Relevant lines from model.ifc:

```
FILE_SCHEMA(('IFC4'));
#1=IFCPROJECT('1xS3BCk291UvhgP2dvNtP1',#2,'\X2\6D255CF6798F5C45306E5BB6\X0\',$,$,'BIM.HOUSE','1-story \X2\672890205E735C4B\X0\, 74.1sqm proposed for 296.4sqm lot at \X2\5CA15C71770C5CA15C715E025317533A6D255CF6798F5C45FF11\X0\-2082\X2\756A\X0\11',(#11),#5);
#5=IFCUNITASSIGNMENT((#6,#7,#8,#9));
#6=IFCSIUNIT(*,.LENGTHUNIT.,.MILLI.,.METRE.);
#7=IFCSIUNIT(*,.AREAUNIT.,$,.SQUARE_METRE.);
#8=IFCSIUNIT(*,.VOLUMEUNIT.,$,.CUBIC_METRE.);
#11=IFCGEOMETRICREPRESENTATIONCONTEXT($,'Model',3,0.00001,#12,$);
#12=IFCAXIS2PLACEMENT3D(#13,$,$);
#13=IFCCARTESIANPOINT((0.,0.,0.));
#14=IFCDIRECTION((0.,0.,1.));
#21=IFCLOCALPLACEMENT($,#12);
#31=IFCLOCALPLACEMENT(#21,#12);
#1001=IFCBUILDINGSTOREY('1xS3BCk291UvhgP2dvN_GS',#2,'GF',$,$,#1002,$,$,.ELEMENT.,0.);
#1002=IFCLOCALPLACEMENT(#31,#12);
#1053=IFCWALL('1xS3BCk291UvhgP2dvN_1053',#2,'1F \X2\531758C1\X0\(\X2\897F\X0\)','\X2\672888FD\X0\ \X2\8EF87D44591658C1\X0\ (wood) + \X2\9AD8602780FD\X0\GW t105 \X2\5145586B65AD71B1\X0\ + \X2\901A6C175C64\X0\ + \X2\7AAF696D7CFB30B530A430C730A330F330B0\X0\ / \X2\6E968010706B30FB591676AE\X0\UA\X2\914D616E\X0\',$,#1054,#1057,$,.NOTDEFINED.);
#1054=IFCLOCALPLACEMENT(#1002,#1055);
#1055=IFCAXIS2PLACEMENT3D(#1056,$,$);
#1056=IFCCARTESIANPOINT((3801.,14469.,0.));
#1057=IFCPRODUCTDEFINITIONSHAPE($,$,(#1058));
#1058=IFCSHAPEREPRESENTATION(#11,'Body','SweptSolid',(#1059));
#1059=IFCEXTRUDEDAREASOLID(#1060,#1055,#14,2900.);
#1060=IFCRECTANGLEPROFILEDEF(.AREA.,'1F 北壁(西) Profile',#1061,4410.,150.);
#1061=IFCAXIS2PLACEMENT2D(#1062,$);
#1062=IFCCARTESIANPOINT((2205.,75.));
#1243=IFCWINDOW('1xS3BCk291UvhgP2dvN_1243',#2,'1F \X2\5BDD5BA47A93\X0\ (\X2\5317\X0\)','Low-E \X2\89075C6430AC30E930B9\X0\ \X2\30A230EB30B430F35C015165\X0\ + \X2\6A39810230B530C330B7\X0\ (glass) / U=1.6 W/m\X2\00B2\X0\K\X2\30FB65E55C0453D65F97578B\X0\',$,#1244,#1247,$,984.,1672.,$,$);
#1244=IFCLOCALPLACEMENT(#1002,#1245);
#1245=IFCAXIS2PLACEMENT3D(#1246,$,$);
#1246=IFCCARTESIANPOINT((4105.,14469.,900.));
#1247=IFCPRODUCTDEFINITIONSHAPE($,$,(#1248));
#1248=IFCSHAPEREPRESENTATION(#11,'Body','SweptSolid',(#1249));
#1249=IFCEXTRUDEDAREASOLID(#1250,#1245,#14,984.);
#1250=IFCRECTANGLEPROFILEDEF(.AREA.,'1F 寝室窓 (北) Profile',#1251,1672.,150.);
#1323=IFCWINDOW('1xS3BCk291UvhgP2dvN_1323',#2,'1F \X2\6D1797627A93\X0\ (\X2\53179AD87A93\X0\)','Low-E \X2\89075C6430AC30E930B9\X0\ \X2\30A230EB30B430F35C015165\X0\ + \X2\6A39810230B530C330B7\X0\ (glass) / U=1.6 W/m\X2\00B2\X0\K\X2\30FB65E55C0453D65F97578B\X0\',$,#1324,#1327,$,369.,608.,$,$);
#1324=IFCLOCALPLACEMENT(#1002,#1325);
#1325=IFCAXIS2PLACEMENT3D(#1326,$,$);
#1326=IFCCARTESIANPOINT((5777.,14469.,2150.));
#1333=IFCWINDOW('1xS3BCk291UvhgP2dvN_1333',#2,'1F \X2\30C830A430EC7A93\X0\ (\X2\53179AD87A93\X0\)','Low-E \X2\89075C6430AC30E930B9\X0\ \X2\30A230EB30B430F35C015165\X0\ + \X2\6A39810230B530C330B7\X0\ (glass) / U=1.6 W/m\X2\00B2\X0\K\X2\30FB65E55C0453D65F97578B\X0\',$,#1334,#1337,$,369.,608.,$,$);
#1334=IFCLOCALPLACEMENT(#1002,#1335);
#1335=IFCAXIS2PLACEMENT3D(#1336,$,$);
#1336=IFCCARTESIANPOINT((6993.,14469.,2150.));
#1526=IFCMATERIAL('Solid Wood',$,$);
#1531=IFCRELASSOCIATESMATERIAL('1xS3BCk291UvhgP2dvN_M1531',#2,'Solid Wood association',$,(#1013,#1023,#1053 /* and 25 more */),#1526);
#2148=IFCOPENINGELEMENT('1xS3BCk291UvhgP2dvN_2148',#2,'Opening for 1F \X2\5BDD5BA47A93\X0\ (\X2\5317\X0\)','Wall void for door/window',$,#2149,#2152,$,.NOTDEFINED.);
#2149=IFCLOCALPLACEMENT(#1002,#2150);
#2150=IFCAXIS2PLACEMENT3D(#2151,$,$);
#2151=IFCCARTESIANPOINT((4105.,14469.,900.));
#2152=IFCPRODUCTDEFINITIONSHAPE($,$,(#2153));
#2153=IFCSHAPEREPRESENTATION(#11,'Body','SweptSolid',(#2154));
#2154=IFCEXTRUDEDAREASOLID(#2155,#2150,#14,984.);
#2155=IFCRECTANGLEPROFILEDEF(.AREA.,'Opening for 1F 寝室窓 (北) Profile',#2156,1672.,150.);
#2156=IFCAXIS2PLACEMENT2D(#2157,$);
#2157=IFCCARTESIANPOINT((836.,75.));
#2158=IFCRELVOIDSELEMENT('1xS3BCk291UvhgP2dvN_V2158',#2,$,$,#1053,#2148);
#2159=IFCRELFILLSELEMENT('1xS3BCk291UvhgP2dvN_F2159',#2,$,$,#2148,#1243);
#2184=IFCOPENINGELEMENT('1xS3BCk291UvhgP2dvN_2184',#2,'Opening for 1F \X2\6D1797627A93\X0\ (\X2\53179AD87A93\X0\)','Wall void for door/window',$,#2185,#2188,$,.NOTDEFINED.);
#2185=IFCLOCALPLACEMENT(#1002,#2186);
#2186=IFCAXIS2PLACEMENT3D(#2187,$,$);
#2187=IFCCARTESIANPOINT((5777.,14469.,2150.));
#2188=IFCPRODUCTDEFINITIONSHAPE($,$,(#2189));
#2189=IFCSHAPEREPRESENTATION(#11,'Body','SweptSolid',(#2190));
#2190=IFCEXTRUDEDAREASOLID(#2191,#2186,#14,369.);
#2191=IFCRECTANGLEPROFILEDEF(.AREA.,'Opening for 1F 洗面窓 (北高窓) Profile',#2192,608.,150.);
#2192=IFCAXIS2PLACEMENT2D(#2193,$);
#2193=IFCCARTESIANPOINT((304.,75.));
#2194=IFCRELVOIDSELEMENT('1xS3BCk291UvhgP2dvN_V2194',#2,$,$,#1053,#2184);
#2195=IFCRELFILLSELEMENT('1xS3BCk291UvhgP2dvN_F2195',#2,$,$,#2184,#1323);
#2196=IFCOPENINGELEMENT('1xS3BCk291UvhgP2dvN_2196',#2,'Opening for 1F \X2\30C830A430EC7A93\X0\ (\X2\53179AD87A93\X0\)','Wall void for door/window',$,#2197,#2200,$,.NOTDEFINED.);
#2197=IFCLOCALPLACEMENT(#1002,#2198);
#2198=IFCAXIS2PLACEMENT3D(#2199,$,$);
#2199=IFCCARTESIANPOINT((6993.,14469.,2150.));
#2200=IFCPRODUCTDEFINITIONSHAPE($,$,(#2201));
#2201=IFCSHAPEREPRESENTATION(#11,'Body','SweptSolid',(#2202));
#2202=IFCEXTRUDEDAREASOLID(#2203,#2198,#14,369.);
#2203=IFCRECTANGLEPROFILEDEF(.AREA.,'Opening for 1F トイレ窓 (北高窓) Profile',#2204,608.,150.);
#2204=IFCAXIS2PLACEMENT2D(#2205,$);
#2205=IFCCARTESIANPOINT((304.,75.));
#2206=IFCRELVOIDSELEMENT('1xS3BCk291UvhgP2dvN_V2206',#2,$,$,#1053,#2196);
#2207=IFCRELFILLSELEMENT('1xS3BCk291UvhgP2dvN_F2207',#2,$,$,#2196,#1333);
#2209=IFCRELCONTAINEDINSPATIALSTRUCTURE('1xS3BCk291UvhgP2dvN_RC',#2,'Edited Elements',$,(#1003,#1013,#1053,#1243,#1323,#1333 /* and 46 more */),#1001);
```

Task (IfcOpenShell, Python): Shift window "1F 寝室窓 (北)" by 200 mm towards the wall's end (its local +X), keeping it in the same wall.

```python
import ifcopenshell
import ifcopenshell.api.geometry
import ifcopenshell.util.placement
import ifcopenshell.util.unit

model = ifcopenshell.open("model.ifc")
unit_scale = ifcopenshell.util.unit.calculate_unit_scale(model)

window = model.by_id(1243)
opening = window.FillsVoids[0].RelatingOpeningElement
wall = opening.VoidsElements[0].RelatingBuildingElement

wall_matrix = ifcopenshell.util.placement.get_local_placement(wall.ObjectPlacement)
shift = wall_matrix[:3, 0] * 0.2 / unit_scale
before = ifcopenshell.util.placement.get_local_placement(window.ObjectPlacement)[:3, 3].copy()

# The window is not placed relative to its opening, so move both.
for product in (opening, window):
    matrix = ifcopenshell.util.placement.get_local_placement(product.ObjectPlacement)
    matrix[:3, 3] += shift
    ifcopenshell.api.geometry.edit_object_placement(model, product=product, matrix=matrix, is_si=False)

after = ifcopenshell.util.placement.get_local_placement(window.ObjectPlacement)[:3, 3]
print("window moved by", (after - before).round(3) + 0.0)

model.write("model_edited.ifc")
```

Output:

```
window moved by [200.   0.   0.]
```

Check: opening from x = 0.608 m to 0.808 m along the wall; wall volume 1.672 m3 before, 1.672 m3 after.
